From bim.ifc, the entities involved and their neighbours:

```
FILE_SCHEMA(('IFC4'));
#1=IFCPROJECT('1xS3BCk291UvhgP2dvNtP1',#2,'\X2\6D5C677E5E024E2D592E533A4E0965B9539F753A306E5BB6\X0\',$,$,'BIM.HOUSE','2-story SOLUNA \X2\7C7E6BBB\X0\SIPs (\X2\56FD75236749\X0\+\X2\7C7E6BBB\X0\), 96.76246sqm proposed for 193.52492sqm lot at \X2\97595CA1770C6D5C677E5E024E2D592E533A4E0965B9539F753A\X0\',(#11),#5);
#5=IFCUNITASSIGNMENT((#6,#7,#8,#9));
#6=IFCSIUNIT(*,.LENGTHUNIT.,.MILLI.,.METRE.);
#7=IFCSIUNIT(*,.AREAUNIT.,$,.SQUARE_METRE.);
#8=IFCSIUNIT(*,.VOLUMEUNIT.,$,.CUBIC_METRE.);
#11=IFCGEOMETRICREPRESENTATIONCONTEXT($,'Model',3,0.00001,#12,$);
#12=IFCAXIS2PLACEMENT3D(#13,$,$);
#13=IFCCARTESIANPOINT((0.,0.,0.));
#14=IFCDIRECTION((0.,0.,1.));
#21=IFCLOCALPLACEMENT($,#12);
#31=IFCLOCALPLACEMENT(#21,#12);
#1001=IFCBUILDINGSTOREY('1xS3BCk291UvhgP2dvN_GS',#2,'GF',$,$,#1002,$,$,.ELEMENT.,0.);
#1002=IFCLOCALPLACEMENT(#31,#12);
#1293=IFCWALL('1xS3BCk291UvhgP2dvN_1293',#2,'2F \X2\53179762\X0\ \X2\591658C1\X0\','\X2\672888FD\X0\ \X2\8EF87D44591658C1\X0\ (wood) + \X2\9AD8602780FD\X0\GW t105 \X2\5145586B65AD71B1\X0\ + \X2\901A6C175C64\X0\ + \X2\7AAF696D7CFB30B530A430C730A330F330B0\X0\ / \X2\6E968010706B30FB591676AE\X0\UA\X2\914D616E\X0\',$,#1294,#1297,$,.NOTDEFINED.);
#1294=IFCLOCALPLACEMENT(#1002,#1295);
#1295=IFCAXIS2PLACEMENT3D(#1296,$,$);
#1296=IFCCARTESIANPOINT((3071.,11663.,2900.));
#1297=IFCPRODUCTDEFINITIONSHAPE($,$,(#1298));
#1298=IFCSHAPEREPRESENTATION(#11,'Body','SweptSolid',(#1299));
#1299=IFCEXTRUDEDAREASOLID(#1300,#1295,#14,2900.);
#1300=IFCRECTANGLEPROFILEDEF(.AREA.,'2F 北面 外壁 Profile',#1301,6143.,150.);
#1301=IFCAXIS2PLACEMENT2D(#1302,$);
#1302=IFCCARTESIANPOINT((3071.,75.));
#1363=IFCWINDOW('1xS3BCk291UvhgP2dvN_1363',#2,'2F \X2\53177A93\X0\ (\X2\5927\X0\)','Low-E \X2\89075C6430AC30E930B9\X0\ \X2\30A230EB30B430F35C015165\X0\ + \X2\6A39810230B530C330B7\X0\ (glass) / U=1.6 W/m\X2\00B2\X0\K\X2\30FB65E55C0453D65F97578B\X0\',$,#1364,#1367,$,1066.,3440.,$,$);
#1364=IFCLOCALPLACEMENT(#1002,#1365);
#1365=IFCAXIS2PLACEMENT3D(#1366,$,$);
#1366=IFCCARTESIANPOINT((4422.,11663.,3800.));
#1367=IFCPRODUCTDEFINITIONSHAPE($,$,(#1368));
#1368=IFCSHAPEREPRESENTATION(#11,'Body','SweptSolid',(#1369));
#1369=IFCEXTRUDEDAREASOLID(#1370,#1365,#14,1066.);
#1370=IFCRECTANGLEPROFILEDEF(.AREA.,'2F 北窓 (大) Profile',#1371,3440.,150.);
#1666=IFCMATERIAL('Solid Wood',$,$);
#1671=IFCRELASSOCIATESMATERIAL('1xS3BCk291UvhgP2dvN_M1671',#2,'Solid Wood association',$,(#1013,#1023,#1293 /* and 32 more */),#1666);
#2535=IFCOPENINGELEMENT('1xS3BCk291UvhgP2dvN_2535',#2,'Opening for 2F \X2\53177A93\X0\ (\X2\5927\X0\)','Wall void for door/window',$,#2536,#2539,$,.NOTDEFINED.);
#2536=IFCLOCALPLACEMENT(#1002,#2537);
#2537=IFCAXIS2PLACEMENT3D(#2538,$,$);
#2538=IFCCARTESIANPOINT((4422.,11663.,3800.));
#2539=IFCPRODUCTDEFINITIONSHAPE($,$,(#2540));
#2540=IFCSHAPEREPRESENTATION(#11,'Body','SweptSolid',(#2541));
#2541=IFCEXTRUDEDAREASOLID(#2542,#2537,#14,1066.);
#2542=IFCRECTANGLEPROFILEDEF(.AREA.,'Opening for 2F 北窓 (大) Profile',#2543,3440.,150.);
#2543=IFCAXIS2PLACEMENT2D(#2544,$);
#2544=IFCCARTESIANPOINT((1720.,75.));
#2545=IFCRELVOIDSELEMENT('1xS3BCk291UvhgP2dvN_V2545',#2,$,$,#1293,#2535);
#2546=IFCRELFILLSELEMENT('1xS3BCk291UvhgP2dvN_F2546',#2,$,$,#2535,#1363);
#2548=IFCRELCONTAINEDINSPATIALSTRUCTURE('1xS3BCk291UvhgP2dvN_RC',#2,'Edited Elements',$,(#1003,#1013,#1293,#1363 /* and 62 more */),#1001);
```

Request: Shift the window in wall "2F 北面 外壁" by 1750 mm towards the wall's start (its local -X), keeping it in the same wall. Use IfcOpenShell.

```python
import ifcopenshell
import ifcopenshell.api.geometry
import ifcopenshell.util.placement
import ifcopenshell.util.unit

model = ifcopenshell.open("bim.ifc")
unit_scale = ifcopenshell.util.unit.calculate_unit_scale(model)

window = model.by_guid("1xS3BCk291UvhgP2dvN_1363")
opening = window.FillsVoids[0].RelatingOpeningElement
wall = opening.VoidsElements[0].RelatingBuildingElement

wall_matrix = ifcopenshell.util.placement.get_local_placement(wall.ObjectPlacement)
shift = wall_matrix[:3, 0] * -1.75 / unit_scale
before = ifcopenshell.util.placement.get_local_placement(window.ObjectPlacement)[:3, 3].copy()

# The window is not placed relative to its opening, so move both.
for product in (opening, window):
    matrix = ifcopenshell.util.placement.get_local_placement(product.ObjectPlacement)
    matrix[:3, 3] += shift
    ifcopenshell.api.geometry.edit_object_placement(model, product=product, matrix=matrix, is_si=False)

after = ifcopenshell.util.placement.get_local_placement(window.ObjectPlacement)[:3, 3]
print("window moved by", (after - before).round(3) + 0.0)

model.write("bim_rev.ifc")
```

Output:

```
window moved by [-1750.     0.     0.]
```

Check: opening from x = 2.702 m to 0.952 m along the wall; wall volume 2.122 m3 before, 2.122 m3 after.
